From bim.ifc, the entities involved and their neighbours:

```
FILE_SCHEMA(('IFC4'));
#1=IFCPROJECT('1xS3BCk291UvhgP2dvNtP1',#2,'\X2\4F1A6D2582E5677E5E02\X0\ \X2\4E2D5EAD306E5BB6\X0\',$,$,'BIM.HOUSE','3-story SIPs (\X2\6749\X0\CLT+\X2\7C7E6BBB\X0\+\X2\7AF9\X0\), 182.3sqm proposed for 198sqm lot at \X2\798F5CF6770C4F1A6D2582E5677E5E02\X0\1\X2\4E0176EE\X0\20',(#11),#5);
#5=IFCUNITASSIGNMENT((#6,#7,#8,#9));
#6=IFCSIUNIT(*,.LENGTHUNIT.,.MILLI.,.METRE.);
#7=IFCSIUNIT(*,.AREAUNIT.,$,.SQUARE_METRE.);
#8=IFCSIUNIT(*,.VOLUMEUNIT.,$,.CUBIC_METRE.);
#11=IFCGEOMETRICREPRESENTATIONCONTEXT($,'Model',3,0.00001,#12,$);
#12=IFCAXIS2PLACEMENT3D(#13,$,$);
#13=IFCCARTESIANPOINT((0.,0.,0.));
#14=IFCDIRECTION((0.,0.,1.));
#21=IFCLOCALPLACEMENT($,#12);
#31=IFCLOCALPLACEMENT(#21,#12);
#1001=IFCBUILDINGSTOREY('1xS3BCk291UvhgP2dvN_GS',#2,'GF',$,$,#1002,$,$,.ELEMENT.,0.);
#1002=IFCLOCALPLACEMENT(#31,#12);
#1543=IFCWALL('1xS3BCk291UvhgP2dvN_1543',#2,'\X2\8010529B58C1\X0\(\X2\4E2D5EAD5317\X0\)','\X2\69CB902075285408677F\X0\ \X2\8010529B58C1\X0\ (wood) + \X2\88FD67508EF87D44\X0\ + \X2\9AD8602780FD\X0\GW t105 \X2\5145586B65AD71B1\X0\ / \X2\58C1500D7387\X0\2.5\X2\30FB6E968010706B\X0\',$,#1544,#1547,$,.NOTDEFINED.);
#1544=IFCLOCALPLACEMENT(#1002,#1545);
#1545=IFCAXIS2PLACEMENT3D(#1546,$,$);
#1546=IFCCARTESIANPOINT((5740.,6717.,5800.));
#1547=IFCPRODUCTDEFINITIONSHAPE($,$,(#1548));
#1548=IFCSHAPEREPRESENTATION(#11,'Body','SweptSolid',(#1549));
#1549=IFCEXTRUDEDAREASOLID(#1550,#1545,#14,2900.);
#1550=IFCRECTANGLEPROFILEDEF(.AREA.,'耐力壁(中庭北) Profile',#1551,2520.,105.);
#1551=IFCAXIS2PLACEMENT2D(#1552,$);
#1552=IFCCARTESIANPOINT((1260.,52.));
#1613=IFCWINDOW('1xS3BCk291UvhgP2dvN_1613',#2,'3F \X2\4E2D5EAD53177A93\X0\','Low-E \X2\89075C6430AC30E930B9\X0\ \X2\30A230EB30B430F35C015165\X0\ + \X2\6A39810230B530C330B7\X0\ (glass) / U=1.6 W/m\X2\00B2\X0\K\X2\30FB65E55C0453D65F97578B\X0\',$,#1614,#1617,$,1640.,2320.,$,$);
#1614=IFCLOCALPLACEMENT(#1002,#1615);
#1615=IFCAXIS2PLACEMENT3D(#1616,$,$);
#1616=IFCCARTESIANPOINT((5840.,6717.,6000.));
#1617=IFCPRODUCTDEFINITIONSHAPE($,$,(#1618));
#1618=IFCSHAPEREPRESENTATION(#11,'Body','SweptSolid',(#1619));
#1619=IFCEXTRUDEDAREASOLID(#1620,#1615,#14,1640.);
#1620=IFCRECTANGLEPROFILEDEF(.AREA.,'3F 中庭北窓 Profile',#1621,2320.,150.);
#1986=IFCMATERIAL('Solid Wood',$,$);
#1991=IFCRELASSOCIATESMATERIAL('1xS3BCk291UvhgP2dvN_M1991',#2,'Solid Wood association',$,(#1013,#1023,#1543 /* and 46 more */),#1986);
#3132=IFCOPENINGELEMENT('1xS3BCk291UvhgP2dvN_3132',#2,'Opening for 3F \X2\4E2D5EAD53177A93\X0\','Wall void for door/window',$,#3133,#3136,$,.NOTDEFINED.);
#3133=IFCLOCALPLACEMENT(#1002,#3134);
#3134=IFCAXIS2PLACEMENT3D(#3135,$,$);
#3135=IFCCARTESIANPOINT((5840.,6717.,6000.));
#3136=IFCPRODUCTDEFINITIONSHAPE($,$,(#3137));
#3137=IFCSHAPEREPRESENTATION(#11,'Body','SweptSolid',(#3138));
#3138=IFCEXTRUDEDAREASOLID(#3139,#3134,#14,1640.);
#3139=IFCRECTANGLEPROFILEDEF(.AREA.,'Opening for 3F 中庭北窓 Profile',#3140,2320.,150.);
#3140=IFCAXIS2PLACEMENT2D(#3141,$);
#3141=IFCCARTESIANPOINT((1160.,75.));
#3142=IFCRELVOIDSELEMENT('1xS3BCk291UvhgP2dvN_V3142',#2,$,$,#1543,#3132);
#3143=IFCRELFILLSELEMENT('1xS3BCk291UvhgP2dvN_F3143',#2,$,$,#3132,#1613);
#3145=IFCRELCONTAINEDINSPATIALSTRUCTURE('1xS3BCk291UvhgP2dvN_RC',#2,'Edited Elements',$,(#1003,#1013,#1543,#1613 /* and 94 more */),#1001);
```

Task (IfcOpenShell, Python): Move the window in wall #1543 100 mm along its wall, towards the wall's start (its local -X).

```python
import ifcopenshell
import ifcopenshell.api.geometry
import ifcopenshell.util.placement
import ifcopenshell.util.unit

model = ifcopenshell.open("bim.ifc")
unit_scale = ifcopenshell.util.unit.calculate_unit_scale(model)

window = model.by_guid("1xS3BCk291UvhgP2dvN_1613")
opening = window.FillsVoids[0].RelatingOpeningElement
wall = opening.VoidsElements[0].RelatingBuildingElement

wall_matrix = ifcopenshell.util.placement.get_local_placement(wall.ObjectPlacement)
shift = wall_matrix[:3, 0] * -0.1 / unit_scale
before = ifcopenshell.util.placement.get_local_placement(window.ObjectPlacement)[:3, 3].copy()

# The window is not placed relative to its opening, so move both.
for product in (opening, window):
    matrix = ifcopenshell.util.placement.get_local_placement(product.ObjectPlacement)
    matrix[:3, 3] += shift
    ifcopenshell.api.geometry.edit_object_placement(model, product=product, matrix=matrix, is_si=False)

after = ifcopenshell.util.placement.get_local_placement(window.ObjectPlacement)[:3, 3]
print("window moved by", (after - before).round(3) + 0.0)

model.write("bim_v2.ifc")
```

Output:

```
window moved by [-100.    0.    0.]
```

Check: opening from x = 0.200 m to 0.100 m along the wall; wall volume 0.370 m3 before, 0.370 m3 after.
